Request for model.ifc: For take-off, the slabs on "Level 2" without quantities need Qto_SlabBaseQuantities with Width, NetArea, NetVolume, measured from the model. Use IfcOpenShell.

First a look at what the model holds.

```python
import ifcopenshell
import ifcopenshell.util.element
import ifcopenshell.util.unit

model = ifcopenshell.open("model.ifc")
print(model.schema)
for unit_type in ("LENGTHUNIT", "AREAUNIT", "VOLUMEUNIT"):
    print(unit_type, ifcopenshell.util.unit.calculate_unit_scale(model, unit_type))
storey = next(s for s in model.by_type("IfcBuildingStorey") if s.Name == "Level 2")
slabs = [e for e in ifcopenshell.util.element.get_decomposition(storey) if e.is_a("IfcSlab")]
for e in sorted(slabs, key=lambda e: e.id()):
    print(e.id(), e.is_a(), e.Name, list(ifcopenshell.util.element.get_psets(e, qtos_only=True)), sep=" | ")
```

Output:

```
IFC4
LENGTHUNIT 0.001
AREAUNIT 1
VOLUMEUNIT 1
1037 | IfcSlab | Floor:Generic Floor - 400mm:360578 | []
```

```python
import ifcopenshell
import ifcopenshell.api.pset
import ifcopenshell.geom
import ifcopenshell.util.element
import ifcopenshell.util.shape
import ifcopenshell.util.unit

model = ifcopenshell.open("model.ifc")
unit_scale = ifcopenshell.util.unit.calculate_unit_scale(model)
area_scale = ifcopenshell.util.unit.calculate_unit_scale(model, "AREAUNIT")
volume_scale = ifcopenshell.util.unit.calculate_unit_scale(model, "VOLUMEUNIT")
settings = ifcopenshell.geom.settings()

storey = next(s for s in model.by_type("IfcBuildingStorey") if s.Name == "Level 2")
slabs = [e for e in ifcopenshell.util.element.get_decomposition(storey) if e.is_a("IfcSlab")]

for e in sorted(slabs, key=lambda e: e.id()):
    if ifcopenshell.util.element.get_psets(e, qtos_only=True, should_inherit=False):
        continue
    # Geometry comes back in metres, in the element's own axes.
    shape = ifcopenshell.geom.create_shape(settings, e)
    values = {
        "Width": ifcopenshell.util.shape.get_z(shape.geometry) / unit_scale,
        "NetArea": ifcopenshell.util.shape.get_footprint_area(shape.geometry) / area_scale,
        "NetVolume": ifcopenshell.util.shape.get_volume(shape.geometry) / volume_scale,
    }
    qto = ifcopenshell.api.pset.add_qto(model, product=e, name="Qto_SlabBaseQuantities")
    ifcopenshell.api.pset.edit_qto(model, qto=qto, properties=values)
    print(e.id(), {k: round(v, 3) for k, v in values.items()})

model.write("model_edited.ifc")
```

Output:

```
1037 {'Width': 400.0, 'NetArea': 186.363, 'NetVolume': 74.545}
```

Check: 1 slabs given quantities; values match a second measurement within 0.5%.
